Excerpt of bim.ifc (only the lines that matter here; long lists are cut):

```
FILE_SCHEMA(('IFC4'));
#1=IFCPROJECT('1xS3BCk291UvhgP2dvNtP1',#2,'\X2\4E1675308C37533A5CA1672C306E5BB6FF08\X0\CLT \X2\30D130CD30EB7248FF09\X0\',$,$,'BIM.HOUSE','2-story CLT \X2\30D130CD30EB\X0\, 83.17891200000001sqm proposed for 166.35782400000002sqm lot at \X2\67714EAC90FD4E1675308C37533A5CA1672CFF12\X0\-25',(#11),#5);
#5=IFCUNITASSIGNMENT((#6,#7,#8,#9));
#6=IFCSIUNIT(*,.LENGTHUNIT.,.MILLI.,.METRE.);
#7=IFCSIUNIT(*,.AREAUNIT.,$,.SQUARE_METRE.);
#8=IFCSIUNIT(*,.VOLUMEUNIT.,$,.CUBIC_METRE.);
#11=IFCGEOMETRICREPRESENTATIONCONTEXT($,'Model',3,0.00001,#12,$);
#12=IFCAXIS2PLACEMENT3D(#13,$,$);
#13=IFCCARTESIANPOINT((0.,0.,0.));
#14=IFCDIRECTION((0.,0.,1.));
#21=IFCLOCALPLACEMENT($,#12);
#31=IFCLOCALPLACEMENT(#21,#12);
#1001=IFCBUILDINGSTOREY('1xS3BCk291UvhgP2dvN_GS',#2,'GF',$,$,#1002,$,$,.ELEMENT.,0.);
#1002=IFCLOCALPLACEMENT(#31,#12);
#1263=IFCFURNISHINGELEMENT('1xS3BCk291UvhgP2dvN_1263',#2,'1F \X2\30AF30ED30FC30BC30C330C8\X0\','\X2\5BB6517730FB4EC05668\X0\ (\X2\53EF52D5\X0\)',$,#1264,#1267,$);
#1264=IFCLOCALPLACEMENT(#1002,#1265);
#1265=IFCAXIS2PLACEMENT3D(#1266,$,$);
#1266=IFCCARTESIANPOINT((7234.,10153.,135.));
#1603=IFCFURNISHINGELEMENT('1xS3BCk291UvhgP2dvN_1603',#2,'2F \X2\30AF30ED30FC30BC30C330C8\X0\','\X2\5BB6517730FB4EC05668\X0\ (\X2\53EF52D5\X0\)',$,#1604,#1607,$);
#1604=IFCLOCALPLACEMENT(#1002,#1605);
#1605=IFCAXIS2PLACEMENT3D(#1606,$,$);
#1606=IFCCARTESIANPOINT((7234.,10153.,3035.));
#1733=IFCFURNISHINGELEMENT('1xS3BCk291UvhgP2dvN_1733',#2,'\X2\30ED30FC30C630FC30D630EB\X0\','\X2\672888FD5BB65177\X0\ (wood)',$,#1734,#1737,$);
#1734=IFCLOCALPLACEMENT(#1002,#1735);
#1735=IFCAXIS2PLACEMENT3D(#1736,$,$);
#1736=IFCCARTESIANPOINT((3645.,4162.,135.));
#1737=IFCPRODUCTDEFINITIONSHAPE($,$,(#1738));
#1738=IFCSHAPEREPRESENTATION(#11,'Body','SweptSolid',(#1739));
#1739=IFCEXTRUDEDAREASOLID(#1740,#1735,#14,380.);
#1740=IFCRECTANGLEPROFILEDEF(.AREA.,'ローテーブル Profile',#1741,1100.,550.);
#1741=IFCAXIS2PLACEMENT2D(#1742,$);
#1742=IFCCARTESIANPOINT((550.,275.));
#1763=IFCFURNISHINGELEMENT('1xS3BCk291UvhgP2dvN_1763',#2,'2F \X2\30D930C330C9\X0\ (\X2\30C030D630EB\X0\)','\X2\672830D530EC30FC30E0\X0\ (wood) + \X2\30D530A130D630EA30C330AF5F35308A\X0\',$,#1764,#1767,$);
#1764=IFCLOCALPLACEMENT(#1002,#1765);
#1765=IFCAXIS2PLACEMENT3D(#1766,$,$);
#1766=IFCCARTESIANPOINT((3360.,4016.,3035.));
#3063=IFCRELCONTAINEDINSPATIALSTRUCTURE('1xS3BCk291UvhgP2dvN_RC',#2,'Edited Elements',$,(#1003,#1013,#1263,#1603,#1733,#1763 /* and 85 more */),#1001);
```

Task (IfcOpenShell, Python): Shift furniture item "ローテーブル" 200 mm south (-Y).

```python
import ifcopenshell
import ifcopenshell.api.geometry
import ifcopenshell.util.placement

model = ifcopenshell.open("bim.ifc")

item = model.by_id(1733)
matrix = ifcopenshell.util.placement.get_local_placement(item.ObjectPlacement)
matrix[1, 3] -= 200.0
ifcopenshell.api.geometry.edit_object_placement(model, product=item, matrix=matrix, is_si=False)

print(ifcopenshell.util.placement.get_local_placement(item.ObjectPlacement).round(3) + 0.0)

model.write("bim_rev.ifc")
```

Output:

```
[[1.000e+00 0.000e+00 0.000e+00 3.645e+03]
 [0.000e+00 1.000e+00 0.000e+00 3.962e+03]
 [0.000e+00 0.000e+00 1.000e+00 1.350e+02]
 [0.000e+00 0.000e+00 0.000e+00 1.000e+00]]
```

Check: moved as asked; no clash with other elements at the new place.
